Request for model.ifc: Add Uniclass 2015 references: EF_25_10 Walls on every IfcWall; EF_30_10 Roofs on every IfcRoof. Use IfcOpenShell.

First a look at what the model holds.

```python
import ifcopenshell

model = ifcopenshell.open("model.ifc")
print(model.schema)
print("classifications:", [c.Name for c in model.by_type("IfcClassification")])
for ifc_class in ("IfcDoor", "IfcRoof", "IfcStair", "IfcWall", "IfcWindow"):
    print(ifc_class, len(model.by_type(ifc_class)))
```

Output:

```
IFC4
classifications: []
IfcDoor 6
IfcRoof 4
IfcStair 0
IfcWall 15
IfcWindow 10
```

```python
import ifcopenshell
import ifcopenshell.api.classification

model = ifcopenshell.open("model.ifc")

system = ifcopenshell.api.classification.add_classification(model, classification="Uniclass 2015")

codes = {
    "IfcWall": ("EF_25_10", "Walls"),
    "IfcRoof": ("EF_30_10", "Roofs"),
}
for ifc_class, (code, name) in codes.items():
    products = model.by_type(ifc_class)
    ifcopenshell.api.classification.add_reference(
        model, products=products, classification=system, identification=code, name=name
    )
    print(code, len(products))

model.write("model-out.ifc")
```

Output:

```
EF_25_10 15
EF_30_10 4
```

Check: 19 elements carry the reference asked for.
